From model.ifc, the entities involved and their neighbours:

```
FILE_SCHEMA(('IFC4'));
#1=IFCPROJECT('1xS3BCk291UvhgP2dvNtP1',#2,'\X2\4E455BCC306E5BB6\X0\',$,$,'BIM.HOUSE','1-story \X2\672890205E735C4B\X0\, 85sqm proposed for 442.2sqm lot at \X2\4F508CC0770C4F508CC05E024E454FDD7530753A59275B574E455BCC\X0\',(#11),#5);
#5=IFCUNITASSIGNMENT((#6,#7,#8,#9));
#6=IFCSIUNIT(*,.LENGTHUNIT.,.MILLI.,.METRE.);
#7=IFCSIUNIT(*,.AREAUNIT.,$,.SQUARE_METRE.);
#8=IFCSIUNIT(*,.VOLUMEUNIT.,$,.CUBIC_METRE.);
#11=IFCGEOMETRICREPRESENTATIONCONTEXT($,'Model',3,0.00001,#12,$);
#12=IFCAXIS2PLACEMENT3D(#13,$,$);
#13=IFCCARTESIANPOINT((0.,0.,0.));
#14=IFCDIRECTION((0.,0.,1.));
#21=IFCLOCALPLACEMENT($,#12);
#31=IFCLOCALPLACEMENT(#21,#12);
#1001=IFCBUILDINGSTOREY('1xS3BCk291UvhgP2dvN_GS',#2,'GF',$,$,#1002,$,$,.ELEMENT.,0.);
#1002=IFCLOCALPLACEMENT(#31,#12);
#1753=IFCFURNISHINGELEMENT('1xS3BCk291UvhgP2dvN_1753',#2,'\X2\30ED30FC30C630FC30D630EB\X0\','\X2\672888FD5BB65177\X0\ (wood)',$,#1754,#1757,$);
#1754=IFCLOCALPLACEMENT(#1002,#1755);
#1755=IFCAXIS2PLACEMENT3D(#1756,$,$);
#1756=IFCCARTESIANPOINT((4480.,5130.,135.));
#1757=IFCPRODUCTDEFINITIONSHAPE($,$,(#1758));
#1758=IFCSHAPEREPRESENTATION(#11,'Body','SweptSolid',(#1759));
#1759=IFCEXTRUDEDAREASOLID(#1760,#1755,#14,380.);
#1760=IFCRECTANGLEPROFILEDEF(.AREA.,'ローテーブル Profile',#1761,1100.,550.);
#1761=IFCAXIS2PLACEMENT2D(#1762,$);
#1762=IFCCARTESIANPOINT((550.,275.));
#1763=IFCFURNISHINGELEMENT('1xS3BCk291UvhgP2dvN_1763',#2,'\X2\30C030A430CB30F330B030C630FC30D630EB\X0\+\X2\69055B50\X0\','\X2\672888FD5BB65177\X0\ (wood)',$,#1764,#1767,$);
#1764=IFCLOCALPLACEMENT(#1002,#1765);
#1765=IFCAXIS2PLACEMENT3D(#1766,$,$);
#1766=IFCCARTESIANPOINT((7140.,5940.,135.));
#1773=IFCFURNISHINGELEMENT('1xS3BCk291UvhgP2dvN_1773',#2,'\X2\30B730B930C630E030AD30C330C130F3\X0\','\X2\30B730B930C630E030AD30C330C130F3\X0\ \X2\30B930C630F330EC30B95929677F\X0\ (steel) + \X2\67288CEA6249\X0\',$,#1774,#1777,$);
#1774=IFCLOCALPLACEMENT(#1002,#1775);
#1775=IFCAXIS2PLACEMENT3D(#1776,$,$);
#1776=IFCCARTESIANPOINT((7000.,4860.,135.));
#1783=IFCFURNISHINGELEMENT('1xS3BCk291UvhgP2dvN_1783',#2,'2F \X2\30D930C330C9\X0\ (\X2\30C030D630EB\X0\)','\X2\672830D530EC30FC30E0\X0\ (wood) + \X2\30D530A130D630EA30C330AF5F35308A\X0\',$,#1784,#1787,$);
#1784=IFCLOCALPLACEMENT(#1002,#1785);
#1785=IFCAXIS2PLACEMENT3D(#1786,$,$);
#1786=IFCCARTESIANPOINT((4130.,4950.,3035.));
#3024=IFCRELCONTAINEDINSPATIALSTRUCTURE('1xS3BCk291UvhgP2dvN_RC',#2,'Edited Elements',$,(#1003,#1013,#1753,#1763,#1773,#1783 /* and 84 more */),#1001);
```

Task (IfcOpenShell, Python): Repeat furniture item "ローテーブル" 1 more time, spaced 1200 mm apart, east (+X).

```python
import numpy as np
import ifcopenshell
import ifcopenshell.api.geometry
import ifcopenshell.api.root
import ifcopenshell.util.element
import ifcopenshell.util.placement
import ifcopenshell.util.unit

model = ifcopenshell.open("model.ifc")
unit_scale = ifcopenshell.util.unit.calculate_unit_scale(model)


def reuse_history(source, copy):
    """copy_class also copies each property set's owner history, people and application; keep the originals."""
    for rel in copy.IsDefinedBy:
        if rel.is_a("IfcRelDefinesByProperties") and (history := rel.RelatingPropertyDefinition.OwnerHistory):
            rel.RelatingPropertyDefinition.OwnerHistory = source.OwnerHistory
            ifcopenshell.util.element.remove_deep2(model, history)


source = model.by_guid("1xS3BCk291UvhgP2dvN_1753")
base = ifcopenshell.util.placement.get_local_placement(source.ObjectPlacement)
step = np.array([1.0, 0.0, 0.0]) * 1.2 / unit_scale

for i in range(1, 2):
    copy = ifcopenshell.api.root.copy_class(model, product=source)
    copy.Representation = ifcopenshell.util.element.copy_deep(
        model, source.Representation, exclude=["IfcGeometricRepresentationContext", "IfcRepresentationMap"]
    )
    reuse_history(source, copy)
    matrix = base.copy()
    matrix[:3, 3] += i * step
    print("added at", matrix[:3, 3].round(3) + 0.0)
    ifcopenshell.api.geometry.edit_object_placement(model, product=copy, matrix=matrix, is_si=False)

model.write("model_updated.ifc")
```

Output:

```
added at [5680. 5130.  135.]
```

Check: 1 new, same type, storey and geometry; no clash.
